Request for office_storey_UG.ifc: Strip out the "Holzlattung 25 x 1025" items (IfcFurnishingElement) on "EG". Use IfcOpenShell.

First a look at what the model holds.

```python
import ifcopenshell
import ifcopenshell.util.element

model = ifcopenshell.open("office_storey_UG.ifc")
print(model.schema)
storey = next(s for s in model.by_type("IfcBuildingStorey") if s.Name == "EG")
furniture = [e for e in ifcopenshell.util.element.get_decomposition(storey) if e.is_a("IfcFurnishingElement")]
seen = {}
for e in furniture:
    element_type = ifcopenshell.util.element.get_type(e)
    name = element_type.Name if element_type not in (None, e) else None
    seen[name] = seen.get(name, 0) + 1
for name, count in sorted(seen.items(), key=str):
    print(count, "x", name)
```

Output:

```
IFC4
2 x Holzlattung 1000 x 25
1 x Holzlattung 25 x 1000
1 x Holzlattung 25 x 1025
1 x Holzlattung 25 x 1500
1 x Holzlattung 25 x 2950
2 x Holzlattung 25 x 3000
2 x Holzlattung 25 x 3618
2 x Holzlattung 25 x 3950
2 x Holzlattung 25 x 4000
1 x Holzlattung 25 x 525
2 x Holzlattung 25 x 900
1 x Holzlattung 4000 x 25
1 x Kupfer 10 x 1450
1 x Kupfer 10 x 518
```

```python
import ifcopenshell
import ifcopenshell.api.root
import ifcopenshell.util.element

model = ifcopenshell.open("office_storey_UG.ifc")

storey = next(s for s in model.by_type("IfcBuildingStorey") if s.Name == "EG")
furniture = [e for e in ifcopenshell.util.element.get_decomposition(storey) if e.is_a("IfcFurnishingElement")]
targets = [e for e in furniture if (t := ifcopenshell.util.element.get_type(e)) not in (None, e) and t.Name == "Holzlattung 25 x 1025"]

for e in targets:
    ifcopenshell.api.root.remove_product(model, product=e)
print(len(targets), "removed")

model.write("office_storey_UG_updated.ifc")
```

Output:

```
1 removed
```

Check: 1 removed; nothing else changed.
